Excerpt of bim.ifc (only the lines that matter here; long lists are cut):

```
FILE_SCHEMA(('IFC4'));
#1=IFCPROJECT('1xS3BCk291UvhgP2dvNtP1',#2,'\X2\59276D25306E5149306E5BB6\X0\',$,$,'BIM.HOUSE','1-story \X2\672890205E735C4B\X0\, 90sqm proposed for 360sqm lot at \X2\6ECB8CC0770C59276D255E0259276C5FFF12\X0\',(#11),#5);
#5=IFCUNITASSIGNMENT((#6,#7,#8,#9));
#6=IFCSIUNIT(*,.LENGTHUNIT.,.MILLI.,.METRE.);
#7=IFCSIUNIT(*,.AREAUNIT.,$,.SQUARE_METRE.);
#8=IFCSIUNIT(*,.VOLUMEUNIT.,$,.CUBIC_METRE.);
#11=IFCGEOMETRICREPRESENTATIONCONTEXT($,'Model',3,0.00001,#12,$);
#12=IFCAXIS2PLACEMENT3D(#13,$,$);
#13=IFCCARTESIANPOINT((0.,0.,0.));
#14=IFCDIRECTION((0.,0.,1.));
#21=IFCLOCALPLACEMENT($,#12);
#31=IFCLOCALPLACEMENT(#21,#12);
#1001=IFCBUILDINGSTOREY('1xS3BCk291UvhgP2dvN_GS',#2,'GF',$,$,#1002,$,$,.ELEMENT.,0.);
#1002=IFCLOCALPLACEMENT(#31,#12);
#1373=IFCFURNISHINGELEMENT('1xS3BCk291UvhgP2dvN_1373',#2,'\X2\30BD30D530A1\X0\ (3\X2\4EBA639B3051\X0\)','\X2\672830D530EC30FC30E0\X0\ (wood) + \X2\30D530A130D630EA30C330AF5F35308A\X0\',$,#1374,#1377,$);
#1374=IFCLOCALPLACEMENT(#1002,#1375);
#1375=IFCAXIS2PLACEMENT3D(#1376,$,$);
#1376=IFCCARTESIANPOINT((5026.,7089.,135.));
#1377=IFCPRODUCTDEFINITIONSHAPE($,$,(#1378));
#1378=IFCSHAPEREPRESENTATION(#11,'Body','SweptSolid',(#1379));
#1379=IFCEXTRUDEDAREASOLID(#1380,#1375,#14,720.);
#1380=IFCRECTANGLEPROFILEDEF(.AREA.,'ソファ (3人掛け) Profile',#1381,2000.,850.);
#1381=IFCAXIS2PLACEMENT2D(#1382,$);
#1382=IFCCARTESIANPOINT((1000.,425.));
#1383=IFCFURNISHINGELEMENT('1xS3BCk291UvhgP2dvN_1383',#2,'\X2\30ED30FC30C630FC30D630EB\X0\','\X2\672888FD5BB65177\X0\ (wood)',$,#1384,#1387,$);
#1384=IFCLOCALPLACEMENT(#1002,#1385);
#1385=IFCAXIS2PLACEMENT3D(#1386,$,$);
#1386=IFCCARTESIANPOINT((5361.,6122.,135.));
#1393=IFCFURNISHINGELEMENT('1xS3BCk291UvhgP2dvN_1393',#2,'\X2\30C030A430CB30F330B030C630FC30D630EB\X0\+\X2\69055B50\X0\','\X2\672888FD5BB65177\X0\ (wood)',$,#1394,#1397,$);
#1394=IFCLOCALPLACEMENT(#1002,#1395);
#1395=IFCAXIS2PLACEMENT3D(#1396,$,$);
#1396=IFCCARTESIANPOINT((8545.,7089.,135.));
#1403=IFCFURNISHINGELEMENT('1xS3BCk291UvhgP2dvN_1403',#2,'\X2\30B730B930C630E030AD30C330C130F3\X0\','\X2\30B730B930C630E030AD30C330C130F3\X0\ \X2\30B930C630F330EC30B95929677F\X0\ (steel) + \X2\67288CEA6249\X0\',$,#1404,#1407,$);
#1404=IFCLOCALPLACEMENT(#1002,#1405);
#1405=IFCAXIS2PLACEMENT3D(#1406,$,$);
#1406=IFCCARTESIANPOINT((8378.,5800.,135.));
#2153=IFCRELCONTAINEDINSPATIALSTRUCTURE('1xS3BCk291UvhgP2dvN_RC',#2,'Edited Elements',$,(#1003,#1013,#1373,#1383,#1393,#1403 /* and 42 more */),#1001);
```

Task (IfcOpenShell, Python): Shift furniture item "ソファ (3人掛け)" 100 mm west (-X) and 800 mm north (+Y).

```python
import ifcopenshell
import ifcopenshell.api.geometry
import ifcopenshell.util.placement
import ifcopenshell.util.unit

model = ifcopenshell.open("bim.ifc")
unit_scale = ifcopenshell.util.unit.calculate_unit_scale(model)

item = model.by_id(1373)
matrix = ifcopenshell.util.placement.get_local_placement(item.ObjectPlacement)
matrix[0, 3] -= 0.1 / unit_scale
matrix[1, 3] += 0.8 / unit_scale
ifcopenshell.api.geometry.edit_object_placement(model, product=item, matrix=matrix, is_si=False)

print(ifcopenshell.util.placement.get_local_placement(item.ObjectPlacement).round(3) + 0.0)

model.write("bim_v2.ifc")
```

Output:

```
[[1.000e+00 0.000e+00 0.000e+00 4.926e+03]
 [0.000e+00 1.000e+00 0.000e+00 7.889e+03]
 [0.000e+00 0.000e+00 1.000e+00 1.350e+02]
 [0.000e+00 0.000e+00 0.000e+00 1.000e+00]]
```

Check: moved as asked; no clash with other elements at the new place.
